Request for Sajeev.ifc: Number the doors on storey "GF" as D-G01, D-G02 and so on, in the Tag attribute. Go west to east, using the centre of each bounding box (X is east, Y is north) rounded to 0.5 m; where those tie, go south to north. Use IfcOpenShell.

First a look at what the model holds.

```python
import ifcopenshell
import ifcopenshell.util.element
import ifcopenshell.util.placement

model = ifcopenshell.open("Sajeev.ifc")
print(model.schema)
storey = next(s for s in model.by_type("IfcBuildingStorey") if s.Name == "GF")
doors = [e for e in ifcopenshell.util.element.get_decomposition(storey) if e.is_a("IfcDoor")]
for e in sorted(doors, key=lambda e: e.id()):
    origin = ifcopenshell.util.placement.get_local_placement(e.ObjectPlacement)[:3, 3]
    print(e.id(), e.Tag, e.Name, origin.round(2) + 0.0, sep=" | ")
```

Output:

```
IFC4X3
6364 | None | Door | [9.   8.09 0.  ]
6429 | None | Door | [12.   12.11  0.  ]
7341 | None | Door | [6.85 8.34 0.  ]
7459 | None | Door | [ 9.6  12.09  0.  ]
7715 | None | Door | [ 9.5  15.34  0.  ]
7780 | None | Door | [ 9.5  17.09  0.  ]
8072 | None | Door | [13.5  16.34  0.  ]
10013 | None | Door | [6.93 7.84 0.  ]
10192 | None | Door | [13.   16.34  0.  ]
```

```python
import ifcopenshell
import ifcopenshell.geom
import ifcopenshell.util.element
import ifcopenshell.util.shape

model = ifcopenshell.open("Sajeev.ifc")
settings = ifcopenshell.geom.settings()
settings.set("use-world-coords", True)


def centre(element):
    shape = ifcopenshell.geom.create_shape(settings, element)
    return ifcopenshell.util.shape.get_bbox_centroid(shape.geometry)


storey = next(s for s in model.by_type("IfcBuildingStorey") if s.Name == "GF")
doors = [e for e in ifcopenshell.util.element.get_decomposition(storey) if e.is_a("IfcDoor")]

# Insertion points can sit at a corner or the storey origin, so sort by the geometry (in metres).
centres = {e: centre(e) for e in doors}
doors.sort(key=lambda e: (round(centres[e][0] / 0.5), centres[e][1]))

for i, e in enumerate(doors, start=1):
    number = f"D-G{i:02d}"
    e.Tag = number
    print(e.id(), number)

model.write("Sajeev_v2.ifc")
```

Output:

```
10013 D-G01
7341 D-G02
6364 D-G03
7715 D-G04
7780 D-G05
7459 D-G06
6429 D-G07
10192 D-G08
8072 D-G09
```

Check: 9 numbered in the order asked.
